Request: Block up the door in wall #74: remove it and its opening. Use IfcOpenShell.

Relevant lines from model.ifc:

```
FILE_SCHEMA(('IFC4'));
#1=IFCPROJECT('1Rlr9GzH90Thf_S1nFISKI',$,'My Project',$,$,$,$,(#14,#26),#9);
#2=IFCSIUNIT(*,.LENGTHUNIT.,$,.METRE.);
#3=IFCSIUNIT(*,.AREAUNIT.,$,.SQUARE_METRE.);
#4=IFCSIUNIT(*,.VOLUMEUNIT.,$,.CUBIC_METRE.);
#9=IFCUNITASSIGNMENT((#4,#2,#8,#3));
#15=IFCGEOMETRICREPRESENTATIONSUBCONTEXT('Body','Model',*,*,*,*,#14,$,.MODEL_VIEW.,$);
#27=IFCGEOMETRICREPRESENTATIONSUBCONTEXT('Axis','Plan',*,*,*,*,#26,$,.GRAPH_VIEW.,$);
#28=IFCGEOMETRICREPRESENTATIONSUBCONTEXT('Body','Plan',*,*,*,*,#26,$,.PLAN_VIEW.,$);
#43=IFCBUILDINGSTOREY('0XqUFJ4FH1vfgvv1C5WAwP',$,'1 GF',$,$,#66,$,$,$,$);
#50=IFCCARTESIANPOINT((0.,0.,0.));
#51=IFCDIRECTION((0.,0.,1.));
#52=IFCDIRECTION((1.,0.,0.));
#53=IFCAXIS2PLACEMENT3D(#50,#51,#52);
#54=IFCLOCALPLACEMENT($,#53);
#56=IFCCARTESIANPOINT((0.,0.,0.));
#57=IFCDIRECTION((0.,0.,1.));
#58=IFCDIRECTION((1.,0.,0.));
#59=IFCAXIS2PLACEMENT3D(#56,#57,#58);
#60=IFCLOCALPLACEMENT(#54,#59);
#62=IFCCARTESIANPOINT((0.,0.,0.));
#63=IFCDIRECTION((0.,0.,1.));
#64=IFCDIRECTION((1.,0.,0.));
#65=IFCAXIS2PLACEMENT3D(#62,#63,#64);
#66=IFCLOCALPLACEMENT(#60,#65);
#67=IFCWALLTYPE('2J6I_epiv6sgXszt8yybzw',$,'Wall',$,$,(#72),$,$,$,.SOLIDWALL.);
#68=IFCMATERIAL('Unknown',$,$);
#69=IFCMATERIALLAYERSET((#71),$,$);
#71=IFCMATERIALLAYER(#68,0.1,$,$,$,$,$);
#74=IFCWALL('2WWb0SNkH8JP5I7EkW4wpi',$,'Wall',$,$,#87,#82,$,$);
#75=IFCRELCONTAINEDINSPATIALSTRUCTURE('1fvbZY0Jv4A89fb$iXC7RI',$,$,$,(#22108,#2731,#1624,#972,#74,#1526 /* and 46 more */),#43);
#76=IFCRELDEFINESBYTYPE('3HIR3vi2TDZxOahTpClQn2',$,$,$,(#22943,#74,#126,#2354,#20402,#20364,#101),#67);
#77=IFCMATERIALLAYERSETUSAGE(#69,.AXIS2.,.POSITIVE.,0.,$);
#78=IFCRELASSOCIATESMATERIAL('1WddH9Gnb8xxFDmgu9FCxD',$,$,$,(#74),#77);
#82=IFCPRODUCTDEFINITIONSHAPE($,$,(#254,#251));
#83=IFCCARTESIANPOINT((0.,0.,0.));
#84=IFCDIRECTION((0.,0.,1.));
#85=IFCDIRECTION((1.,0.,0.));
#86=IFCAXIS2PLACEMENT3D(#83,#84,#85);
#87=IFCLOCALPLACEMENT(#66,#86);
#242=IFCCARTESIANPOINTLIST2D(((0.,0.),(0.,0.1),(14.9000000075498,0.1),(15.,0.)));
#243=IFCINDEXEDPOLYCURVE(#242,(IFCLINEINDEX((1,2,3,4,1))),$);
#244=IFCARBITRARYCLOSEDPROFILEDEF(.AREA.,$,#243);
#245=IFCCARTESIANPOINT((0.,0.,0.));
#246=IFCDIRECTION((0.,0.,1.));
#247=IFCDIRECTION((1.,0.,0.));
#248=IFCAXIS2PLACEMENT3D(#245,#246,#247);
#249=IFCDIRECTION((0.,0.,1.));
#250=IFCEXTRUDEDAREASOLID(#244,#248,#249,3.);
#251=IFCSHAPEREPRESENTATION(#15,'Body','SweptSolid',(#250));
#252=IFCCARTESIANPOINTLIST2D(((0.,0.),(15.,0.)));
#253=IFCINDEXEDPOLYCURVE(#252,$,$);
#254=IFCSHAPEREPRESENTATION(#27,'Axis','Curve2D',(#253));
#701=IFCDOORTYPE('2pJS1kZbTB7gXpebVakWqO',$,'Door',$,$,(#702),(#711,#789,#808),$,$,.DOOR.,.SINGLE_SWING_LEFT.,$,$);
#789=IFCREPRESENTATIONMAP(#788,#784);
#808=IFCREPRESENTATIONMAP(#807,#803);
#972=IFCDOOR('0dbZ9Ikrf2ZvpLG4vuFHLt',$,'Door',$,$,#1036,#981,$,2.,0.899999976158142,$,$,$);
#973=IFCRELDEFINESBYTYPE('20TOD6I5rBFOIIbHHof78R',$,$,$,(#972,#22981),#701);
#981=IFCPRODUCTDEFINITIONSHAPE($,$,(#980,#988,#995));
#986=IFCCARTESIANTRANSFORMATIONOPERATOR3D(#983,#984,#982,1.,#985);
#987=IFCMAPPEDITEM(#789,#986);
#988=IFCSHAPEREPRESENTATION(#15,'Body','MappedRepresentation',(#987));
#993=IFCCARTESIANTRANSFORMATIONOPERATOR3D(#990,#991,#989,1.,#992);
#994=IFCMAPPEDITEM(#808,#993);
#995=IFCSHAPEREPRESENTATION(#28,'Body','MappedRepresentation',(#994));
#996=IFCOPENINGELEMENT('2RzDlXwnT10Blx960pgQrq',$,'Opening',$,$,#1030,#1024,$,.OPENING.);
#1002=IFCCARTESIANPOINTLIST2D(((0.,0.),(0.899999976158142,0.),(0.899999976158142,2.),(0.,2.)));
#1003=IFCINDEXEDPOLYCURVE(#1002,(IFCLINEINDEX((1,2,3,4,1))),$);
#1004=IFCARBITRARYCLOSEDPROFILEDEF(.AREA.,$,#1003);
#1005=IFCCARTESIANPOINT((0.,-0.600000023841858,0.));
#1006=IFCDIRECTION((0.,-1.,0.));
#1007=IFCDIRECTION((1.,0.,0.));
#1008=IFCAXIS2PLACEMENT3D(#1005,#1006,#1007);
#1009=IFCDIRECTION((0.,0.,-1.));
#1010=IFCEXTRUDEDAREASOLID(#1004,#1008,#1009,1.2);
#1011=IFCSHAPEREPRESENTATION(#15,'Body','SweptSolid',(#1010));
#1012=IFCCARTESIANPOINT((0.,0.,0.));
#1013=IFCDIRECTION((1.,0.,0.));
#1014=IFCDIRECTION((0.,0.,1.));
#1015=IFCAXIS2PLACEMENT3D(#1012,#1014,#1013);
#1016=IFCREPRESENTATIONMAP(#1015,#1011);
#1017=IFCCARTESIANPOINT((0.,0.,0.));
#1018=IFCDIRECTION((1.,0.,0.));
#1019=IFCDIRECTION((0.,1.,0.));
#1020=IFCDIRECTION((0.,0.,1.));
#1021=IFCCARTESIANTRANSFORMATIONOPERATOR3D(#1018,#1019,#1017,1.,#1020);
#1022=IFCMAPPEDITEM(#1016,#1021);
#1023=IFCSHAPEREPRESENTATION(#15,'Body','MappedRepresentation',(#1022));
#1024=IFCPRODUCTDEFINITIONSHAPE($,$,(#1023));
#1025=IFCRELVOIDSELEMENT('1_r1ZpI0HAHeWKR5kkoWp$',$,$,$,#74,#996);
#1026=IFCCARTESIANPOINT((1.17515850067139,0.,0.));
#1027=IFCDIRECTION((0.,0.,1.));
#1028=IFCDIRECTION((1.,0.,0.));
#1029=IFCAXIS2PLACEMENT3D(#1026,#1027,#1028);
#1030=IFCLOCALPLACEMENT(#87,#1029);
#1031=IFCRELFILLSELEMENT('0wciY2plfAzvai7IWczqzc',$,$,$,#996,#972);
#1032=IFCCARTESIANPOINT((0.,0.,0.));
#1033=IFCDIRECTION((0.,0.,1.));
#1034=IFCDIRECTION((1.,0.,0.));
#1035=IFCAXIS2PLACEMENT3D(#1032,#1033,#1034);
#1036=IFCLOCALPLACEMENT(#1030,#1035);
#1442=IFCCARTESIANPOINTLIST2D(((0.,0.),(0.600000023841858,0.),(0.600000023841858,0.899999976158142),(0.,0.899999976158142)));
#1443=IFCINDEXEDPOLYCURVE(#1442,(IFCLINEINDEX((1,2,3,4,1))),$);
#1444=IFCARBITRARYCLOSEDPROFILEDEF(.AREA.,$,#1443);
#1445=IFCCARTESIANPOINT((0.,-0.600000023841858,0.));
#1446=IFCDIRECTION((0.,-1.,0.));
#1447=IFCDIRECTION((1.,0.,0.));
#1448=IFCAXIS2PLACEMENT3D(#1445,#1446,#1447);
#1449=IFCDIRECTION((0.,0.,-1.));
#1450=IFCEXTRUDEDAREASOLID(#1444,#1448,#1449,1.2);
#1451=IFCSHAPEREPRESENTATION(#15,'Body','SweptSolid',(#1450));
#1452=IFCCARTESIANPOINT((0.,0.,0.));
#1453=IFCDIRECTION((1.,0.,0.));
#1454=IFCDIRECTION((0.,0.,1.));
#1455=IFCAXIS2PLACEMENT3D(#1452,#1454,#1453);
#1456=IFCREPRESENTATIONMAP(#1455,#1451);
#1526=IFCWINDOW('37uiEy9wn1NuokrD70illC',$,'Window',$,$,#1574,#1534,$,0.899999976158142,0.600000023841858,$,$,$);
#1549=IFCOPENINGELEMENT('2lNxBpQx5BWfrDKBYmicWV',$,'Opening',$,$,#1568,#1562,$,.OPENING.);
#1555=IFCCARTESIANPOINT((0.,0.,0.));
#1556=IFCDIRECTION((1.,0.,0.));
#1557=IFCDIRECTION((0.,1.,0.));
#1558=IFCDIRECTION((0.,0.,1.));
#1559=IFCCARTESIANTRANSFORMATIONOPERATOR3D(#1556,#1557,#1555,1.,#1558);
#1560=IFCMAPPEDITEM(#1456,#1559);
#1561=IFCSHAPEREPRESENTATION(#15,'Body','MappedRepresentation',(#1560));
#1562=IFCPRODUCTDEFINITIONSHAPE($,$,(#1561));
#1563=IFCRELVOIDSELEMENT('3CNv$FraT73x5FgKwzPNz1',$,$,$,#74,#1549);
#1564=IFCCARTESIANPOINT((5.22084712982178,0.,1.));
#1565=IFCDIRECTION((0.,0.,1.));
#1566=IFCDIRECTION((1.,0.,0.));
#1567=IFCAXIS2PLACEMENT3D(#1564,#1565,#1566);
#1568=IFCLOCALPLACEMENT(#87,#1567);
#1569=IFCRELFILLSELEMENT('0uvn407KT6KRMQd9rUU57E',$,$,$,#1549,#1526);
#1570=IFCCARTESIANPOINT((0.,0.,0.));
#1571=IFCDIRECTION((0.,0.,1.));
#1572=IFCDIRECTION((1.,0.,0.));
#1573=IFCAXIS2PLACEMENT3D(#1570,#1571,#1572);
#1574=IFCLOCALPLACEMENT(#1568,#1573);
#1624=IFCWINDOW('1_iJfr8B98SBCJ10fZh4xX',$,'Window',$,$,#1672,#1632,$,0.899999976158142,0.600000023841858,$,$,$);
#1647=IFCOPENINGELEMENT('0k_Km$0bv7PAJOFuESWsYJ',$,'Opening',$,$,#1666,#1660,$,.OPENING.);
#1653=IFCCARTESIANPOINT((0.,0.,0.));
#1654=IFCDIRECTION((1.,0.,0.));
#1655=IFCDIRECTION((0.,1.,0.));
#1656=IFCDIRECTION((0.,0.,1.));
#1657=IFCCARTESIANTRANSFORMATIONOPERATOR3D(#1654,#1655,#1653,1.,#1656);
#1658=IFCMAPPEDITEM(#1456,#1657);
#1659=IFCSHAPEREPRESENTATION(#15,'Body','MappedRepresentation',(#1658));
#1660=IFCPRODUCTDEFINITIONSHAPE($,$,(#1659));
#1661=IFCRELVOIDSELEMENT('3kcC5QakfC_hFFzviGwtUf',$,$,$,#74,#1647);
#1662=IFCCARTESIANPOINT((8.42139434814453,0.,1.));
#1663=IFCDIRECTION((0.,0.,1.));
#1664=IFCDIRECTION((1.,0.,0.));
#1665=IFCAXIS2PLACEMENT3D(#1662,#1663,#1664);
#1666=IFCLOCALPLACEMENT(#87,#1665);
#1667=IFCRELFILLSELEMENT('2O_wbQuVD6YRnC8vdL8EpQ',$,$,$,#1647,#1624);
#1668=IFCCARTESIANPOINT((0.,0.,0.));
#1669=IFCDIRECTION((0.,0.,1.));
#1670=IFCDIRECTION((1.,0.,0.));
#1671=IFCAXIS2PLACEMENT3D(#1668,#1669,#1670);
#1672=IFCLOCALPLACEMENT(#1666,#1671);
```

```python
import ifcopenshell
import ifcopenshell.api.feature
import ifcopenshell.api.root
import ifcopenshell.geom
import ifcopenshell.util.shape

model = ifcopenshell.open("model.ifc")
settings = ifcopenshell.geom.settings()


def volume(element):
    """Net volume in cubic metres, openings subtracted."""
    shape = ifcopenshell.geom.create_shape(settings, element)
    return ifcopenshell.util.shape.get_volume(shape.geometry)


door = model.by_guid("0dbZ9Ikrf2ZvpLG4vuFHLt")
opening = door.FillsVoids[0].RelatingOpeningElement
wall = opening.VoidsElements[0].RelatingBuildingElement
before = volume(wall)

ifcopenshell.api.root.remove_product(model, product=door)
ifcopenshell.api.feature.remove_feature(model, feature=opening)

after = volume(wall)

print(f"wall volume {before:.3f} -> {after:.3f} m3")

model.write("model_edited.ifc")
```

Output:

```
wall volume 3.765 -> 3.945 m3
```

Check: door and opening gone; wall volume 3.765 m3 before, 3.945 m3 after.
